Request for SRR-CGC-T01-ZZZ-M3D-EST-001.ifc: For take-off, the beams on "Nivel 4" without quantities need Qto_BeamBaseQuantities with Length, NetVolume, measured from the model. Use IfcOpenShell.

First a look at what the model holds.

```python
import ifcopenshell
import ifcopenshell.util.element
import ifcopenshell.util.unit

model = ifcopenshell.open("SRR-CGC-T01-ZZZ-M3D-EST-001.ifc")
print(model.schema)
for unit_type in ("LENGTHUNIT", "AREAUNIT", "VOLUMEUNIT"):
    print(unit_type, ifcopenshell.util.unit.calculate_unit_scale(model, unit_type))
storey = next(s for s in model.by_type("IfcBuildingStorey") if s.Name == "Nivel 4")
beams = [e for e in ifcopenshell.util.element.get_decomposition(storey) if e.is_a("IfcBeam")]
for e in sorted(beams, key=lambda e: e.id()):
    print(e.id(), e.is_a(), e.Name, list(ifcopenshell.util.element.get_psets(e, qtos_only=True)), sep=" | ")
```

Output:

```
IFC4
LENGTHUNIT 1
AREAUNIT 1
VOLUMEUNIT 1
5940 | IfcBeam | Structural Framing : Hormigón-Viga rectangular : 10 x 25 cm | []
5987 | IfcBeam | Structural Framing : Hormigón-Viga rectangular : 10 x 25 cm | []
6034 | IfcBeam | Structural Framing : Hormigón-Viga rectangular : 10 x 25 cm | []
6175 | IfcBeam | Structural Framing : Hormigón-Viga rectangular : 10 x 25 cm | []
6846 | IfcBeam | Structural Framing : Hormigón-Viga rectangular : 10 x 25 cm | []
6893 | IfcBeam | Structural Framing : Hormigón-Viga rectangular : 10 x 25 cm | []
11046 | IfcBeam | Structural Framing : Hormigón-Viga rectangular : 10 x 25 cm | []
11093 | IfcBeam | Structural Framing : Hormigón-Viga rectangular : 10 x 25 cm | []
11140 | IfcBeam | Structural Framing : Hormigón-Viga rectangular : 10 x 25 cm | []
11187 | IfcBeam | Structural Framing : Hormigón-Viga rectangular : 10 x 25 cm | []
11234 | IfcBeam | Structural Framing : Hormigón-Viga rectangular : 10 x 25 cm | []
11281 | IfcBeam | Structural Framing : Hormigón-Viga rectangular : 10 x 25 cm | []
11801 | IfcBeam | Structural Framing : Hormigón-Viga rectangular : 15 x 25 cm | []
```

```python
import ifcopenshell
import ifcopenshell.api.pset
import ifcopenshell.geom
import ifcopenshell.util.element
import ifcopenshell.util.shape
import ifcopenshell.util.unit

model = ifcopenshell.open("SRR-CGC-T01-ZZZ-M3D-EST-001.ifc")
unit_scale = ifcopenshell.util.unit.calculate_unit_scale(model)
volume_scale = ifcopenshell.util.unit.calculate_unit_scale(model, "VOLUMEUNIT")
settings = ifcopenshell.geom.settings()

storey = next(s for s in model.by_type("IfcBuildingStorey") if s.Name == "Nivel 4")
beams = [e for e in ifcopenshell.util.element.get_decomposition(storey) if e.is_a("IfcBeam")]

for e in sorted(beams, key=lambda e: e.id()):
    if ifcopenshell.util.element.get_psets(e, qtos_only=True, should_inherit=False):
        continue
    # Geometry comes back in metres, in the element's own axes.
    shape = ifcopenshell.geom.create_shape(settings, e)
    values = {
        "Length": ifcopenshell.util.shape.get_max_xyz(shape.geometry) / unit_scale,
        "NetVolume": ifcopenshell.util.shape.get_volume(shape.geometry) / volume_scale,
    }
    qto = ifcopenshell.api.pset.add_qto(model, product=e, name="Qto_BeamBaseQuantities")
    ifcopenshell.api.pset.edit_qto(model, qto=qto, properties=values)
    print(e.id(), {k: round(v, 3) for k, v in values.items()})

model.write("SRR-CGC-T01-ZZZ-M3D-EST-001_rev.ifc")
```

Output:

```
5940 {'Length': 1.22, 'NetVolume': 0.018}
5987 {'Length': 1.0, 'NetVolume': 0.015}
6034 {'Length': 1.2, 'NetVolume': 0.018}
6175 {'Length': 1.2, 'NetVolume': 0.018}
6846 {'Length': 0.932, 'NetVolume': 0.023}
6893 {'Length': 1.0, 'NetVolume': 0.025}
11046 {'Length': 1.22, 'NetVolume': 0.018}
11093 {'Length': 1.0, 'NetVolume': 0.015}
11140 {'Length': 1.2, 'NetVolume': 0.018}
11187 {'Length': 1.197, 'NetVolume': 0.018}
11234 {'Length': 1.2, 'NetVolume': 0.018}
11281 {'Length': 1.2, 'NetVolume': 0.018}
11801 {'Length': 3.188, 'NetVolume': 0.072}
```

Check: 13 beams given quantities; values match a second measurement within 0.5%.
